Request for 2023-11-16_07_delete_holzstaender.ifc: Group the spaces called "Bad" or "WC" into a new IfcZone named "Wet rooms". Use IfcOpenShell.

First a look at what the model holds.

```python
import ifcopenshell

model = ifcopenshell.open("2023-11-16_07_delete_holzstaender.ifc")
print(model.schema)
seen = {}
for space in model.by_type("IfcSpace"):
    seen[space.LongName] = seen.get(space.LongName, 0) + 1
for name, count in sorted(seen.items(), key=str):
    print(count, "x", name)
print("zones:", [z.Name for z in model.by_type("IfcZone")][:20])
```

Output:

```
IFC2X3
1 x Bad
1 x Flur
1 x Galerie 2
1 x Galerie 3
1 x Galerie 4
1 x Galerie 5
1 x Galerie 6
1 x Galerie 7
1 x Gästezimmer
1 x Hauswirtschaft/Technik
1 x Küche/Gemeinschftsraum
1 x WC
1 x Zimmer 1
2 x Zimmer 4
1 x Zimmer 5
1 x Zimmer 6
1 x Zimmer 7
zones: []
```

```python
import ifcopenshell
import ifcopenshell.api.group
import ifcopenshell.api.root

model = ifcopenshell.open("2023-11-16_07_delete_holzstaender.ifc")

names = {"Bad", "WC"}
spaces = [s for s in model.by_type("IfcSpace") if s.LongName in names]

zone = ifcopenshell.api.root.create_entity(model, ifc_class="IfcZone", name="Wet rooms")
ifcopenshell.api.group.assign_group(model, products=spaces, group=zone)
print(len(spaces), "spaces in", zone.Name)

model.write("2023-11-16_07_delete_holzstaender_updated.ifc")
```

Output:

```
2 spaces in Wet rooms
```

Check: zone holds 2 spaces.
